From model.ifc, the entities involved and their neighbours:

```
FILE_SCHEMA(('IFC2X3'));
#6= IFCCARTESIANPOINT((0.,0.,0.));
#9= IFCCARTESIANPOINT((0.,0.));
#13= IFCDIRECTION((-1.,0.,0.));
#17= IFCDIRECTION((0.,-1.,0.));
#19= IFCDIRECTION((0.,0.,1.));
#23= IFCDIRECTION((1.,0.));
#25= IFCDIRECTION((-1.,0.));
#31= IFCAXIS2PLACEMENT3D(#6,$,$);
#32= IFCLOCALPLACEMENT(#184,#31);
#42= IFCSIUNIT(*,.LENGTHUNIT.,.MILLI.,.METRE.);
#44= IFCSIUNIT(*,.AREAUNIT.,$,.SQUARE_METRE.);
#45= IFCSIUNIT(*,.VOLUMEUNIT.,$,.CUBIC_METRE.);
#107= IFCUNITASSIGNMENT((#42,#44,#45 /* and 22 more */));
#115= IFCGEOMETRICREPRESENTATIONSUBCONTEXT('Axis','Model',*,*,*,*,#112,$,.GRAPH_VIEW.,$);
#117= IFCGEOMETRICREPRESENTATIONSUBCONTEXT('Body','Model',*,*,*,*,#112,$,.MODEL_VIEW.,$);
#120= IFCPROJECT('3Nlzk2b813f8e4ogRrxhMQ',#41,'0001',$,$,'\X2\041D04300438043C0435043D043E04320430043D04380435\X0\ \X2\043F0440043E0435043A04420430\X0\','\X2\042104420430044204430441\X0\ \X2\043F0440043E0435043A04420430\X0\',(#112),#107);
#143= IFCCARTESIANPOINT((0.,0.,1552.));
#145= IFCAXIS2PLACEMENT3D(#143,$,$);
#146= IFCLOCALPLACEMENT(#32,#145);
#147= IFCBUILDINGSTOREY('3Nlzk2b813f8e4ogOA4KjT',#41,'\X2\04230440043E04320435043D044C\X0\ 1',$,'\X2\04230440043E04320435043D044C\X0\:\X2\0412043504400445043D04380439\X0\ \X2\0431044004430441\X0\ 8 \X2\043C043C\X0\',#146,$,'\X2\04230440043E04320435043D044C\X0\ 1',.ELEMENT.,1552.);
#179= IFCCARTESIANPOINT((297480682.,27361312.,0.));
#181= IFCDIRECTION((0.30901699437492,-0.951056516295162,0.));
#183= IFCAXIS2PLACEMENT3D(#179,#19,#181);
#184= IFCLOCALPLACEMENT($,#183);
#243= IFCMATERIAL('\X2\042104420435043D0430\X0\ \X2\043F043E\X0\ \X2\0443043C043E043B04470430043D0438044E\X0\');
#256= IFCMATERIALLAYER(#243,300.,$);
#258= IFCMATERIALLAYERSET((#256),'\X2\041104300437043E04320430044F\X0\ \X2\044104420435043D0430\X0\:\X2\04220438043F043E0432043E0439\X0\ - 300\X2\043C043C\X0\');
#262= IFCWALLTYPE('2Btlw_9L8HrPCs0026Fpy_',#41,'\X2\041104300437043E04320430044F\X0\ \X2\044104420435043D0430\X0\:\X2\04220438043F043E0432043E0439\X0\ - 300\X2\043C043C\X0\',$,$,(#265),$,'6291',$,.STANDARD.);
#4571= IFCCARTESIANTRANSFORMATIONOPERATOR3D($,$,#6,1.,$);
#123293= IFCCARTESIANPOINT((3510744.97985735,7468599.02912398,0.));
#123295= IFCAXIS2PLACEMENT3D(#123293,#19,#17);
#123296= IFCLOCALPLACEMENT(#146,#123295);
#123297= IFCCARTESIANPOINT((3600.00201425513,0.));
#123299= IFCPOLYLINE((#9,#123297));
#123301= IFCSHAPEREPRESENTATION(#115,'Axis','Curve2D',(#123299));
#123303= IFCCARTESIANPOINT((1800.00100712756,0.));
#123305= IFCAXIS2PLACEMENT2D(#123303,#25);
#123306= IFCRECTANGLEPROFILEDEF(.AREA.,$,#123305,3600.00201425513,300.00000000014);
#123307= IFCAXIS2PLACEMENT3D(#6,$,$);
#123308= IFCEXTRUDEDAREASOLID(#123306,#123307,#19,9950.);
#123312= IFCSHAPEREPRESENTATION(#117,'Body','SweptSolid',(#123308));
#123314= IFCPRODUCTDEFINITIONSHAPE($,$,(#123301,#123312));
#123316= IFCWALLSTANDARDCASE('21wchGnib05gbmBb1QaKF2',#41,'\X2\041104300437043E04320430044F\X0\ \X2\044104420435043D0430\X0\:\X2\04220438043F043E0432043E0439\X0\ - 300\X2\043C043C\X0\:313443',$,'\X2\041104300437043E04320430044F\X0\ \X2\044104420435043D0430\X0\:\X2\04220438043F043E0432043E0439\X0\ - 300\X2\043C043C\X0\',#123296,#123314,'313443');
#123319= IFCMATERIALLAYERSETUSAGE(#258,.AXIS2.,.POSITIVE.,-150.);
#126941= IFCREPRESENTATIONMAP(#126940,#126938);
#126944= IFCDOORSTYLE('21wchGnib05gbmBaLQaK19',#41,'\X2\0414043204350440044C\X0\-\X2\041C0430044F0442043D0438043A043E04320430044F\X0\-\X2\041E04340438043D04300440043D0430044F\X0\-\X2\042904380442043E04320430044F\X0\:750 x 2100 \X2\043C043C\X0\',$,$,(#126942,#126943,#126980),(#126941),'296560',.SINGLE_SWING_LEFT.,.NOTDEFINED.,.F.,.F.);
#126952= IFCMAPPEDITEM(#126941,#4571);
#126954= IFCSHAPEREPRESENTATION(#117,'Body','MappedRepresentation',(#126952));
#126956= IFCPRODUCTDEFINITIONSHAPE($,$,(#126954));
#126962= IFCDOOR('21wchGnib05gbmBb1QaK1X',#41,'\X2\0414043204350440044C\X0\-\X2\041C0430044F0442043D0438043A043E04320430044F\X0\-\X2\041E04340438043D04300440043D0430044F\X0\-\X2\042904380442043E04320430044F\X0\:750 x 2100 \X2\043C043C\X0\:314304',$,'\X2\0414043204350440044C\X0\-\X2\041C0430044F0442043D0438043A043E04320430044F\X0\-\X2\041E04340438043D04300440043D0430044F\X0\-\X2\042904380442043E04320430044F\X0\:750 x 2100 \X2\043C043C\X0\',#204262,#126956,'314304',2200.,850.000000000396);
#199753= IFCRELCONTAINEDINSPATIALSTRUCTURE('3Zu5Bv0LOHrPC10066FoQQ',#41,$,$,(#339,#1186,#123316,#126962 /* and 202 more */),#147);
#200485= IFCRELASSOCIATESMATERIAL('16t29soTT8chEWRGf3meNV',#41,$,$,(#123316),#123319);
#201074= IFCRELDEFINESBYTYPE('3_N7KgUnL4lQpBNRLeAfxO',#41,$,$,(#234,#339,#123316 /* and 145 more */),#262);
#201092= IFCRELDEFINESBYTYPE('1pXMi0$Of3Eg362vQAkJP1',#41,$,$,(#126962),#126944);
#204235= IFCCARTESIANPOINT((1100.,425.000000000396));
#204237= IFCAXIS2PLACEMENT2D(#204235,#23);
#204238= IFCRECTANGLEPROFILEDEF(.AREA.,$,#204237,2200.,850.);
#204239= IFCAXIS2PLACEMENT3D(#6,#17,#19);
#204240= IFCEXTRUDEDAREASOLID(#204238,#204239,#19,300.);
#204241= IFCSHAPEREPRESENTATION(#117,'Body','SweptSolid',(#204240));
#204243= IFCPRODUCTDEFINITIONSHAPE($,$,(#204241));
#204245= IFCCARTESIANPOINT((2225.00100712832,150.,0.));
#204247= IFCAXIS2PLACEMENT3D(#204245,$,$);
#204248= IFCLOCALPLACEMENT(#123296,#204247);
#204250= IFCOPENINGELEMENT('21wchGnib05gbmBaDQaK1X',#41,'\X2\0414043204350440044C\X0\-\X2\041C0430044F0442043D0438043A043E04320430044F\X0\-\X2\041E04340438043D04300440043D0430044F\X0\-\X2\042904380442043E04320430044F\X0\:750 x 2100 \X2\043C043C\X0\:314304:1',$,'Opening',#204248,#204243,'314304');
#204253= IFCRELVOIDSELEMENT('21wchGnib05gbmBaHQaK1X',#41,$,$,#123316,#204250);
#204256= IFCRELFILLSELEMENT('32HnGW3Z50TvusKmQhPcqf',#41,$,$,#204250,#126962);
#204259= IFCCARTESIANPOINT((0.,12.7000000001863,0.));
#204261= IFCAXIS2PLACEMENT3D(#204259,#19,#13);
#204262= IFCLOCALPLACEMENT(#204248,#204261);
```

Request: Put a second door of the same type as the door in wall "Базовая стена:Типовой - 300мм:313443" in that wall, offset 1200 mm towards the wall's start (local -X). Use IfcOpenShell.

```python
import ifcopenshell
import ifcopenshell.api.feature
import ifcopenshell.api.geometry
import ifcopenshell.api.root
import ifcopenshell.geom
import ifcopenshell.util.element
import ifcopenshell.util.placement
import ifcopenshell.util.shape

model = ifcopenshell.open("model.ifc")
settings = ifcopenshell.geom.settings()


def volume(element):
    """Net volume in cubic metres, openings subtracted."""
    shape = ifcopenshell.geom.create_shape(settings, element)
    return ifcopenshell.util.shape.get_volume(shape.geometry)


def reuse_history(source, copy):
    """copy_class also copies each property set's owner history, people and application; keep the originals."""
    for rel in copy.IsDefinedBy:
        if rel.is_a("IfcRelDefinesByProperties") and (history := rel.RelatingPropertyDefinition.OwnerHistory):
            rel.RelatingPropertyDefinition.OwnerHistory = source.OwnerHistory
            ifcopenshell.util.element.remove_deep2(model, history)


door = model.by_id(126962)
opening = door.FillsVoids[0].RelatingOpeningElement
wall = opening.VoidsElements[0].RelatingBuildingElement
before = volume(wall)
shift = ifcopenshell.util.placement.get_local_placement(wall.ObjectPlacement)[:3, 0] * -1200.0

# copy_class copies the void relationship, type, container and properties, but no geometry.
new_opening = ifcopenshell.api.root.copy_class(model, product=opening)
new_opening.Representation = ifcopenshell.util.element.copy_deep(
    model, opening.Representation, exclude=["IfcGeometricRepresentationContext", "IfcRepresentationMap"]
)
new_opening.Name = "Дверь-Маятниковая-Одинарная-Щитовая:750 x 2100 мм"
new_opening.Tag = None
new_door = ifcopenshell.api.root.copy_class(model, product=door)
new_door.Representation = ifcopenshell.util.element.copy_deep(
    model, door.Representation, exclude=["IfcGeometricRepresentationContext", "IfcRepresentationMap"]
)
new_door.Name = "Дверь-Маятниковая-Одинарная-Щитовая:750 x 2100 мм"
new_door.Tag = None
reuse_history(door, new_door)
fills = ifcopenshell.api.feature.add_filling(model, opening=new_opening, element=new_door)
fills.OwnerHistory = new_door.OwnerHistory  # required in IFC2X3

for old, new in ((opening, new_opening), (door, new_door)):
    matrix = ifcopenshell.util.placement.get_local_placement(old.ObjectPlacement)
    matrix[:3, 3] += shift
    ifcopenshell.api.geometry.edit_object_placement(model, product=new, matrix=matrix, is_si=False)

after = volume(wall)

print(f"wall volume {before:.3f} -> {after:.3f} m3")

model.write("model_v2.ifc")
```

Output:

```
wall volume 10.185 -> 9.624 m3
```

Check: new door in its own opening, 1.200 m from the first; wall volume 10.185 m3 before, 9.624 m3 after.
